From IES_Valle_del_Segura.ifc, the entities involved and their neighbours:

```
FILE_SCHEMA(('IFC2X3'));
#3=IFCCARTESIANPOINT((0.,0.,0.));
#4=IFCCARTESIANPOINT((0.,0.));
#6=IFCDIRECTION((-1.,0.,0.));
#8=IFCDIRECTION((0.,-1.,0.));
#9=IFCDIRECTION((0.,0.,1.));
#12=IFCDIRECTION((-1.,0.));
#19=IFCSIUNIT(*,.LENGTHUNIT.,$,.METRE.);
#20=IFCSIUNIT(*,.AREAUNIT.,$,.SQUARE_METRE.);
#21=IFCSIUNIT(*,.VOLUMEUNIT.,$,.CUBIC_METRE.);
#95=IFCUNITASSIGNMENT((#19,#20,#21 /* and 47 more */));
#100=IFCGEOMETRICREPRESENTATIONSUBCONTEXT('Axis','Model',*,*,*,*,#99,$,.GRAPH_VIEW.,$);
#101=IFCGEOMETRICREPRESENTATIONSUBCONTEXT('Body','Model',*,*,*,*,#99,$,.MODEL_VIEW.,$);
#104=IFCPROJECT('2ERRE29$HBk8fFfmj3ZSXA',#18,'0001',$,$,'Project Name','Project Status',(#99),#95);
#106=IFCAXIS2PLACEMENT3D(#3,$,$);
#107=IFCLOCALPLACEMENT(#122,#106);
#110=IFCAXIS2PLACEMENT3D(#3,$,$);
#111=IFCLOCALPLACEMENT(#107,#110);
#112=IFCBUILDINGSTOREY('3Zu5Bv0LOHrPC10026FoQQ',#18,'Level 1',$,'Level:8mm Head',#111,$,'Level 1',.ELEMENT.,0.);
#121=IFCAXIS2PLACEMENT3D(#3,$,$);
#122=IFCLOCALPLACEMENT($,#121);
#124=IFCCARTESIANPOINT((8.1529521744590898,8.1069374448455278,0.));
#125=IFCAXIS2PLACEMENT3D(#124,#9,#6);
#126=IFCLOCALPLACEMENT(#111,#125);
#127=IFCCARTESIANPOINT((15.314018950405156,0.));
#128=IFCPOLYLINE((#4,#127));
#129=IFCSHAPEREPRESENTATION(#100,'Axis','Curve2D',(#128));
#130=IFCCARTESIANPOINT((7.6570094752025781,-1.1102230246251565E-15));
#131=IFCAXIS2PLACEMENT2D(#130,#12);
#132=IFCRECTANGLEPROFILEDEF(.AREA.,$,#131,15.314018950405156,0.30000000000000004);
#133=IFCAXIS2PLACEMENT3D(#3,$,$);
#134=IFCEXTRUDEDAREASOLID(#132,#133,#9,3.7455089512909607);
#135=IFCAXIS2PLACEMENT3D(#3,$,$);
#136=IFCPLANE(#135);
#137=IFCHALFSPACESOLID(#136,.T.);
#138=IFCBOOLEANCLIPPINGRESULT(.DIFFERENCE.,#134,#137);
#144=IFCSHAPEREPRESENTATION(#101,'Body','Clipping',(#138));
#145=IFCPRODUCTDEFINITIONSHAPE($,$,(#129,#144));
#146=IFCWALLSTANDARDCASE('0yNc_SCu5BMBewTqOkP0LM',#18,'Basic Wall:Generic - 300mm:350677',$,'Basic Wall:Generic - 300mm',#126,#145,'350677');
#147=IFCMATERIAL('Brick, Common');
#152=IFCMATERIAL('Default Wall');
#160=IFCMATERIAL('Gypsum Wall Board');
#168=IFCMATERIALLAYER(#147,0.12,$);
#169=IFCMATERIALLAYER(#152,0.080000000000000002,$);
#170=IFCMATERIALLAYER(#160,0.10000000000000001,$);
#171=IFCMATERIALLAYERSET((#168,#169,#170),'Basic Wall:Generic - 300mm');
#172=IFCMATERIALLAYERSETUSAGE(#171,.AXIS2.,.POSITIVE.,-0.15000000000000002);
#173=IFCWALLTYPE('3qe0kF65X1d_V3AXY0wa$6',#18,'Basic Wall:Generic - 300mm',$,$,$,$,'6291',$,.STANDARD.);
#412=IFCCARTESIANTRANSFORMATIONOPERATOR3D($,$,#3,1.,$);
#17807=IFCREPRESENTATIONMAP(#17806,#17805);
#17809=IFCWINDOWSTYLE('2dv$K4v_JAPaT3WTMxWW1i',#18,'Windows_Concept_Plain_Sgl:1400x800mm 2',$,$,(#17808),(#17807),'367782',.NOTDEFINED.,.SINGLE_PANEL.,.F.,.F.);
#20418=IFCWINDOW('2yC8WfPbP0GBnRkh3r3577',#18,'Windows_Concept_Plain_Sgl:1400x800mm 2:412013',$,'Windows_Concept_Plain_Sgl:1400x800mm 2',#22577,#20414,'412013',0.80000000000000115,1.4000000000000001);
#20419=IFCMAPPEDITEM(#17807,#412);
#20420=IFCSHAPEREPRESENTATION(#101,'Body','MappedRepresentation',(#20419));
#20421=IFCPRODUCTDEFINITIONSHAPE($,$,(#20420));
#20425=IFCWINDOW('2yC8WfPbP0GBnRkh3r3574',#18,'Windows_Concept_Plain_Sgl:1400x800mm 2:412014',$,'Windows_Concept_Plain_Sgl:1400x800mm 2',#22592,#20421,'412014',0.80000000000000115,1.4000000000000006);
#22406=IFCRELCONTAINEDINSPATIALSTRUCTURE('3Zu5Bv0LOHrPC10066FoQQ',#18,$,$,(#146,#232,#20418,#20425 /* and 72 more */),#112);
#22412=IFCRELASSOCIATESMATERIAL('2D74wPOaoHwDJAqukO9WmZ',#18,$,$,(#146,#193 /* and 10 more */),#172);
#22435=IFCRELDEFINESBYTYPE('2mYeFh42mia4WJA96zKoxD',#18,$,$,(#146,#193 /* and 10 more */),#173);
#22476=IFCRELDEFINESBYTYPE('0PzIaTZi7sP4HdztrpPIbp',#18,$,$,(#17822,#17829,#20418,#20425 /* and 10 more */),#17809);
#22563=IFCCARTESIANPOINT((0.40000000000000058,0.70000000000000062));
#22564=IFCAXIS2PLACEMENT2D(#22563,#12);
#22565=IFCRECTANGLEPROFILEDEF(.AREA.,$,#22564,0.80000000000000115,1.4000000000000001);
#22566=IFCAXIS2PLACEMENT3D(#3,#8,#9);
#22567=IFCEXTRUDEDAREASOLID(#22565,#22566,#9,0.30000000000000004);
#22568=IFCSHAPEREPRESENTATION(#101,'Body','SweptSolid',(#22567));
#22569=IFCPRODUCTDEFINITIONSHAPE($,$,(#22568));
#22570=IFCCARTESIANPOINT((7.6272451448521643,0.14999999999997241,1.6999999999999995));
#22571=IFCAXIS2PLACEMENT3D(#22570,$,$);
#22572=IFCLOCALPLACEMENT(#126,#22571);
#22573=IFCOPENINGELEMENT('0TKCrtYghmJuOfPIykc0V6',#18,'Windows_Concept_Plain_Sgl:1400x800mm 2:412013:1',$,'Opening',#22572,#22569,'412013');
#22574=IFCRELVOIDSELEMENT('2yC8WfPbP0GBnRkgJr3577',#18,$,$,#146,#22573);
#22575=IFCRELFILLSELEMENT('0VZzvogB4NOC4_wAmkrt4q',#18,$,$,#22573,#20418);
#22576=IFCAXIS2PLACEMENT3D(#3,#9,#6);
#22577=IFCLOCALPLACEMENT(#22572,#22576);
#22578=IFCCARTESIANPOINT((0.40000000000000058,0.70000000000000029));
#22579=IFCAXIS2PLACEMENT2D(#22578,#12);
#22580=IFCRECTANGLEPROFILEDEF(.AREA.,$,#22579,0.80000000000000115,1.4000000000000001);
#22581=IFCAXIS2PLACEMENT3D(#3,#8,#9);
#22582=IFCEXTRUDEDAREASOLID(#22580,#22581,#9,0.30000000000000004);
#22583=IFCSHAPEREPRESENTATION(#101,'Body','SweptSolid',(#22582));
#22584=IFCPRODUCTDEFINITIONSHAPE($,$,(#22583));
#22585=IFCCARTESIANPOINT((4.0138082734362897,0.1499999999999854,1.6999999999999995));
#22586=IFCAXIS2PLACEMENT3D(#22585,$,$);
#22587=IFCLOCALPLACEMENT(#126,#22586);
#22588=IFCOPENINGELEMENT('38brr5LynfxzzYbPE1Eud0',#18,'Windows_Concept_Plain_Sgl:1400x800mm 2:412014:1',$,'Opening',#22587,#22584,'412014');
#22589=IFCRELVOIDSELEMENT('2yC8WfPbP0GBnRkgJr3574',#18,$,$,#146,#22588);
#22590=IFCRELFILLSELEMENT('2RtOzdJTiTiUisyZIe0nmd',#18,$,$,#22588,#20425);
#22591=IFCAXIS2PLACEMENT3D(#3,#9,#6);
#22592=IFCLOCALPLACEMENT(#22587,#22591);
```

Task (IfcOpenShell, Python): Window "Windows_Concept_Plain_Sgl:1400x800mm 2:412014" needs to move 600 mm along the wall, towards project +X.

```python
import ifcopenshell
import ifcopenshell.api.geometry
import ifcopenshell.util.placement
import ifcopenshell.util.unit

model = ifcopenshell.open("IES_Valle_del_Segura.ifc")
unit_scale = ifcopenshell.util.unit.calculate_unit_scale(model)

window = model.by_id(20425)
opening = window.FillsVoids[0].RelatingOpeningElement
wall = opening.VoidsElements[0].RelatingBuildingElement

wall_matrix = ifcopenshell.util.placement.get_local_placement(wall.ObjectPlacement)
shift = wall_matrix[:3, 0] * -0.6 / unit_scale
before = ifcopenshell.util.placement.get_local_placement(window.ObjectPlacement)[:3, 3].copy()

# The window is placed relative to its opening, so it follows when the opening moves.
matrix = ifcopenshell.util.placement.get_local_placement(opening.ObjectPlacement)
matrix[:3, 3] += shift
ifcopenshell.api.geometry.edit_object_placement(
    model, product=opening, matrix=matrix, is_si=False, should_transform_children=True
)

after = ifcopenshell.util.placement.get_local_placement(window.ObjectPlacement)[:3, 3]
print("window moved by", (after - before).round(3) + 0.0)

model.write("IES_Valle_del_Segura_v2.ifc")
```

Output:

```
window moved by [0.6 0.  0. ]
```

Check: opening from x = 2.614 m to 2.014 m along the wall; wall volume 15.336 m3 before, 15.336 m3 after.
